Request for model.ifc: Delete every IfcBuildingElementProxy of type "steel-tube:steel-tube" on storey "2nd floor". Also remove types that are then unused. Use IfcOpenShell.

First a look at what the model holds.

```python
import ifcopenshell
import ifcopenshell.util.element

model = ifcopenshell.open("model.ifc")
print(model.schema)
storey = next(s for s in model.by_type("IfcBuildingStorey") if s.Name == "2nd floor")
proxies = [e for e in ifcopenshell.util.element.get_decomposition(storey) if e.is_a("IfcBuildingElementProxy")]
seen = {}
for e in proxies:
    element_type = ifcopenshell.util.element.get_type(e)
    name = element_type.Name if element_type not in (None, e) else None
    seen[name] = seen.get(name, 0) + 1
for name, count in sorted(seen.items(), key=str):
    print(count, "x", name)
```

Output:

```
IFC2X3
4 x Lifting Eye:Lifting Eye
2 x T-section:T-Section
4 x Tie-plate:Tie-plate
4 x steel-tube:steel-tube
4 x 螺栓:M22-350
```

```python
import ifcopenshell
import ifcopenshell.api.root
import ifcopenshell.util.element

model = ifcopenshell.open("model.ifc")

storey = next(s for s in model.by_type("IfcBuildingStorey") if s.Name == "2nd floor")
proxies = [e for e in ifcopenshell.util.element.get_decomposition(storey) if e.is_a("IfcBuildingElementProxy")]
targets = [e for e in proxies if (t := ifcopenshell.util.element.get_type(e)) not in (None, e) and t.Name == "steel-tube:steel-tube"]
types = {ifcopenshell.util.element.get_type(e) for e in targets} - {None, *targets}

for e in targets:
    ifcopenshell.api.root.remove_product(model, product=e)
print(len(targets), "removed")

unused = [t for t in types if not ifcopenshell.util.element.get_types(t)]
for t in unused:
    ifcopenshell.api.root.remove_product(model, product=t)
print(len(unused), "unused types removed")

model.write("model_updated.ifc")
```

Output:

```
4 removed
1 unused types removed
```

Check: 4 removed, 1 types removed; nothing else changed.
